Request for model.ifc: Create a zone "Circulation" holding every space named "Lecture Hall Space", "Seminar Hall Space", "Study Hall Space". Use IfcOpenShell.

First a look at what the model holds.

```python
import ifcopenshell

model = ifcopenshell.open("model.ifc")
print(model.schema)
seen = {}
for space in model.by_type("IfcSpace"):
    seen[space.LongName] = seen.get(space.LongName, 0) + 1
for name, count in sorted(seen.items(), key=str):
    print(count, "x", name)
print("zones:", [z.Name for z in model.by_type("IfcZone")][:20])
```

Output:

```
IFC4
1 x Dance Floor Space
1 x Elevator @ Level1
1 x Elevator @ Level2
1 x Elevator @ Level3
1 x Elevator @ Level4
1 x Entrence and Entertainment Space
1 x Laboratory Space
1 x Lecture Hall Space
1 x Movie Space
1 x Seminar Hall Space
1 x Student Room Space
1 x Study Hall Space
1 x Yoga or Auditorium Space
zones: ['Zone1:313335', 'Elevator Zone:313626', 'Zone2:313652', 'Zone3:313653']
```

```python
import ifcopenshell
import ifcopenshell.api.group
import ifcopenshell.api.root

model = ifcopenshell.open("model.ifc")

names = {"Lecture Hall Space", "Seminar Hall Space", "Study Hall Space"}
spaces = [s for s in model.by_type("IfcSpace") if s.LongName in names]

zone = ifcopenshell.api.root.create_entity(model, ifc_class="IfcZone", name="Circulation")
ifcopenshell.api.group.assign_group(model, products=spaces, group=zone)
print(len(spaces), "spaces in", zone.Name)

model.write("model_rev.ifc")
```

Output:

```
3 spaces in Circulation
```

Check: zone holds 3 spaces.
